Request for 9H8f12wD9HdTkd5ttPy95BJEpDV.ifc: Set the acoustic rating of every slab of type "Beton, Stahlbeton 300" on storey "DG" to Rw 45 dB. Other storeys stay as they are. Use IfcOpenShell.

First a look at what the model holds.

```python
import ifcopenshell
import ifcopenshell.util.element

model = ifcopenshell.open("9H8f12wD9HdTkd5ttPy95BJEpDV.ifc")
print(model.schema)
storey = next(s for s in model.by_type("IfcBuildingStorey") if s.Name == "DG")
slabs = [e for e in ifcopenshell.util.element.get_decomposition(storey) if e.is_a("IfcSlab")]
seen = {}
for e in slabs:
    element_type = ifcopenshell.util.element.get_type(e)
    key = (element_type.Name if element_type != e and element_type else None, ifcopenshell.util.element.get_pset(e, "Pset_SlabCommon", "AcousticRating"))
    seen[key] = seen.get(key, 0) + 1
for (name, value), count in sorted(seen.items(), key=str):
    print(count, "x", name, "|", value)
```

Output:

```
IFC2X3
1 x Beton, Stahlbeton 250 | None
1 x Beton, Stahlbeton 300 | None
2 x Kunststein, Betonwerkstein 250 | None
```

```python
import ifcopenshell
import ifcopenshell.api.pset
import ifcopenshell.util.element

model = ifcopenshell.open("9H8f12wD9HdTkd5ttPy95BJEpDV.ifc")

storey = next(s for s in model.by_type("IfcBuildingStorey") if s.Name == "DG")
slabs = [e for e in ifcopenshell.util.element.get_decomposition(storey) if e.is_a("IfcSlab")]

count = 0
for e in slabs:
    element_type = ifcopenshell.util.element.get_type(e)
    if element_type in (None, e) or element_type.Name != "Beton, Stahlbeton 300":
        continue
    # add_pset returns the element's existing set when there is one.
    pset = ifcopenshell.api.pset.add_pset(model, product=e, name="Pset_SlabCommon")
    ifcopenshell.api.pset.edit_pset(model, pset=pset, properties={"AcousticRating": "Rw 45 dB"})
    count += 1

print(count, "slabs updated")

model.write("9H8f12wD9HdTkd5ttPy95BJEpDV_v2.ifc")
```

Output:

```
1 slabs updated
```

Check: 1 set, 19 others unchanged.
